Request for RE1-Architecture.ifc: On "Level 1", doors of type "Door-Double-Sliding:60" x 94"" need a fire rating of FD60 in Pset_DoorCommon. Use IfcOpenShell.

First a look at what the model holds.

```python
import ifcopenshell
import ifcopenshell.util.element

model = ifcopenshell.open("RE1-Architecture.ifc")
print(model.schema)
storey = next(s for s in model.by_type("IfcBuildingStorey") if s.Name == "Level 1")
doors = [e for e in ifcopenshell.util.element.get_decomposition(storey) if e.is_a("IfcDoor")]
seen = {}
for e in doors:
    element_type = ifcopenshell.util.element.get_type(e)
    key = (element_type.Name if element_type != e and element_type else None, ifcopenshell.util.element.get_pset(e, "Pset_DoorCommon", "FireRating"))
    seen[key] = seen.get(key, 0) + 1
for (name, value), count in sorted(seen.items(), key=str):
    print(count, "x", name, "|", value)
```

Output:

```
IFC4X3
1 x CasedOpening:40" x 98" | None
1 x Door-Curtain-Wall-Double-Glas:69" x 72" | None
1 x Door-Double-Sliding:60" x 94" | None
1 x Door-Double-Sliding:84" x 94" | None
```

```python
import ifcopenshell
import ifcopenshell.api.pset
import ifcopenshell.util.element

model = ifcopenshell.open("RE1-Architecture.ifc")

storey = next(s for s in model.by_type("IfcBuildingStorey") if s.Name == "Level 1")
doors = [e for e in ifcopenshell.util.element.get_decomposition(storey) if e.is_a("IfcDoor")]

count = 0
for e in doors:
    element_type = ifcopenshell.util.element.get_type(e)
    if element_type in (None, e) or element_type.Name != 'Door-Double-Sliding:60" x 94"':
        continue
    # add_pset returns the element's existing set when there is one.
    pset = ifcopenshell.api.pset.add_pset(model, product=e, name="Pset_DoorCommon")
    ifcopenshell.api.pset.edit_pset(model, pset=pset, properties={"FireRating": "FD60"})
    count += 1

print(count, "doors updated")

model.write("RE1-Architecture_v2.ifc")
```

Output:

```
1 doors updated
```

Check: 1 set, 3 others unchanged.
